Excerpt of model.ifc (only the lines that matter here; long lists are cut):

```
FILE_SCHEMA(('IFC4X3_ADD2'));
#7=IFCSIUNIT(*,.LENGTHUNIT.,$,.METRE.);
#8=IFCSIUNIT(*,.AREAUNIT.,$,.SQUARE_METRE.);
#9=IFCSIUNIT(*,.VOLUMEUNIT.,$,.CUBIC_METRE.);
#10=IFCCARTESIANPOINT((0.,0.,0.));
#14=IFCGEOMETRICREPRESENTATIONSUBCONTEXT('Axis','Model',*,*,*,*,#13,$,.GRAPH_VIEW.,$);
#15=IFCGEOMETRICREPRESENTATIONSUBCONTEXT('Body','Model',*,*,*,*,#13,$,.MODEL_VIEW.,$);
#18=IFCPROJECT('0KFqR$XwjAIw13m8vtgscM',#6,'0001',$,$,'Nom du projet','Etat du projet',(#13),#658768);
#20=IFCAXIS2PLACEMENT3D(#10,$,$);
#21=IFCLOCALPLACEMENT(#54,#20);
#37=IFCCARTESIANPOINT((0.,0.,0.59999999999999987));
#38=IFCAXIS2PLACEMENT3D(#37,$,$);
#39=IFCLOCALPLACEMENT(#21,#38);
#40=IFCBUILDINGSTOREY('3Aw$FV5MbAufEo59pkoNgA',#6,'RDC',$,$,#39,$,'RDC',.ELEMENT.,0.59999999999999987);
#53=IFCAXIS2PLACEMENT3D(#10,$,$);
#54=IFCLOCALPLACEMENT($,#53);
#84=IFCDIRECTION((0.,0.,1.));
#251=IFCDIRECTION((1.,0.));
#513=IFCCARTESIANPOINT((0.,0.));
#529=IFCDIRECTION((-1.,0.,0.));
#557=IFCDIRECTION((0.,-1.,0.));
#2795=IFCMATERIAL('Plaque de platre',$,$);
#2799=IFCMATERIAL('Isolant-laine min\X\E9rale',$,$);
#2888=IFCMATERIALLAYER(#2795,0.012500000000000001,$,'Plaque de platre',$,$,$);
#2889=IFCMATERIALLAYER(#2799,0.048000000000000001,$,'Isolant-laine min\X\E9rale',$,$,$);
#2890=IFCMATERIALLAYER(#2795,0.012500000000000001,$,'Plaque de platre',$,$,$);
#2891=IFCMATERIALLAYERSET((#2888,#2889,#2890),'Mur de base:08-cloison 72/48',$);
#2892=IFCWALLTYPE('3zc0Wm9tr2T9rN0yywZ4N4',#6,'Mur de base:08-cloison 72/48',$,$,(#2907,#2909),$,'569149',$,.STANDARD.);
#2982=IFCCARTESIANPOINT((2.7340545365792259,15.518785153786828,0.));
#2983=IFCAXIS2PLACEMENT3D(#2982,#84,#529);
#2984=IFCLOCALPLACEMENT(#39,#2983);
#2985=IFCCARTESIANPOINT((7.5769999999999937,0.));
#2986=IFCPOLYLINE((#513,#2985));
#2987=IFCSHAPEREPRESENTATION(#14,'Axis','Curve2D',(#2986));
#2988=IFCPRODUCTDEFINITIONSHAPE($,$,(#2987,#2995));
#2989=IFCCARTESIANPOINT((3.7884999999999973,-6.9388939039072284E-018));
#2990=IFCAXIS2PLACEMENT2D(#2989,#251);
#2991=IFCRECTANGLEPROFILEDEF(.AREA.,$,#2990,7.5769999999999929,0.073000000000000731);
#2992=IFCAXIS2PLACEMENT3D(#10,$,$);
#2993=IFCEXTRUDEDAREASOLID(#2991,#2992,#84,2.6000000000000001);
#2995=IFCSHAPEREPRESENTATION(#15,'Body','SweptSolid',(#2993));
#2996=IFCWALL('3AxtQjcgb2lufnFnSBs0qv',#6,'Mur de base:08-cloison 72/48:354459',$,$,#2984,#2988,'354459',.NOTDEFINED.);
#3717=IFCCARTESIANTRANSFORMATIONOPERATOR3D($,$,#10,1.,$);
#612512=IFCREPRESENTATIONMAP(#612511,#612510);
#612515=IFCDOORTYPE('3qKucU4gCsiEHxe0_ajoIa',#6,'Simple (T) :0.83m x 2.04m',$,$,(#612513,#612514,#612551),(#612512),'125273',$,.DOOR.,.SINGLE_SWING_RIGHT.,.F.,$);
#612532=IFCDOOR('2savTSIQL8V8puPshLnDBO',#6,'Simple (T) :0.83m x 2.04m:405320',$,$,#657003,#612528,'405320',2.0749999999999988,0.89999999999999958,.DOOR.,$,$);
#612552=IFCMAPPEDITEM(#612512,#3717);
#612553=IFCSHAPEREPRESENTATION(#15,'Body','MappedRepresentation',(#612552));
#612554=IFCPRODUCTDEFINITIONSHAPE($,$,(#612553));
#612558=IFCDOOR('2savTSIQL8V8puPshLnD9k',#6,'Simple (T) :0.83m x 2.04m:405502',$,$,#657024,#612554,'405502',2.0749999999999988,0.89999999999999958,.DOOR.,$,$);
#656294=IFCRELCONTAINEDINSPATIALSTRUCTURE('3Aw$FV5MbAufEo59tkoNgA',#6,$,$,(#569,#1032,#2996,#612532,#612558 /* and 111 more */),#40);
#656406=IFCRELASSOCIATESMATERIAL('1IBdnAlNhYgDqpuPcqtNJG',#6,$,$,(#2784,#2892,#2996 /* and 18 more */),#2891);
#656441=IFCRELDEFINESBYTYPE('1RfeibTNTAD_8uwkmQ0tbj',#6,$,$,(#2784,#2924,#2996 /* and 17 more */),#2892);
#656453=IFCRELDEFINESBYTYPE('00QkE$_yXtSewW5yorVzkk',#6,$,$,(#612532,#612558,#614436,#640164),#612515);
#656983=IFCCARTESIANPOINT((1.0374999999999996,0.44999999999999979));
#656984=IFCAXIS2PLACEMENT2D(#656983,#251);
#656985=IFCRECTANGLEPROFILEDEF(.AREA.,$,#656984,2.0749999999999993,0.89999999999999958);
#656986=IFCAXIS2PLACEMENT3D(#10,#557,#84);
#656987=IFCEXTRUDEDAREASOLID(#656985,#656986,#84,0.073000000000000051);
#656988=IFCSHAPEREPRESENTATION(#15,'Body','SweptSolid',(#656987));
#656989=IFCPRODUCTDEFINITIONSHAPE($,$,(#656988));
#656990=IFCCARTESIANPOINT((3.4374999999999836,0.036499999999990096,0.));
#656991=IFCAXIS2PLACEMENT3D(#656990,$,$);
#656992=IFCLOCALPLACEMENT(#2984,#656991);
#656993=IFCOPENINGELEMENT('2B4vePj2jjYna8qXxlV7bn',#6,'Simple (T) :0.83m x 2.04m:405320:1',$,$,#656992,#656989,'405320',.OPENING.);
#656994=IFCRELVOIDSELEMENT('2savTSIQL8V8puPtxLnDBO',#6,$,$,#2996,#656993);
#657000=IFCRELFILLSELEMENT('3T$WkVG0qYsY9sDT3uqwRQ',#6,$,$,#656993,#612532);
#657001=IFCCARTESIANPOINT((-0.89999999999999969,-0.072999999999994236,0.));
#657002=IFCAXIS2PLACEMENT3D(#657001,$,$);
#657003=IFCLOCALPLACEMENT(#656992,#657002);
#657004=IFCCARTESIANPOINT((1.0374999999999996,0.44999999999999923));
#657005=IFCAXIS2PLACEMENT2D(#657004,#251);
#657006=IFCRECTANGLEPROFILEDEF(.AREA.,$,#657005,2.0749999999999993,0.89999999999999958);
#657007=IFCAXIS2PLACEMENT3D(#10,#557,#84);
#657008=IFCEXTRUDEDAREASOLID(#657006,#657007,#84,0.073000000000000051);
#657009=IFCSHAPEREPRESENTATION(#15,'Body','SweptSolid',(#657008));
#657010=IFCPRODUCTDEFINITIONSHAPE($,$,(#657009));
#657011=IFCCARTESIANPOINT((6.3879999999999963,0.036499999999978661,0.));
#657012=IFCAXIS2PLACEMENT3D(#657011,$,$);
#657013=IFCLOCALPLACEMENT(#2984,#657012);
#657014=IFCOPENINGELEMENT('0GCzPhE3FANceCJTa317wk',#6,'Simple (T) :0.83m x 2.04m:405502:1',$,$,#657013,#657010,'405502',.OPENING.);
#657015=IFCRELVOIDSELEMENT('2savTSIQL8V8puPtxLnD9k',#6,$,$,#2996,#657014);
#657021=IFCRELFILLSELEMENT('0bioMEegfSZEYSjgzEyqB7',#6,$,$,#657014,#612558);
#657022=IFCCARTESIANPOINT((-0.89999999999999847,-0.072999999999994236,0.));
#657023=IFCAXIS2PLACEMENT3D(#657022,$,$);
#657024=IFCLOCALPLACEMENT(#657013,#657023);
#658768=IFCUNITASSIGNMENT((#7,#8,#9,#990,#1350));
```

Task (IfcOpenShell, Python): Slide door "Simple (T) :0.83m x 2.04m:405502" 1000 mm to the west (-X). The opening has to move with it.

```python
import ifcopenshell
import ifcopenshell.api.geometry
import ifcopenshell.util.placement

model = ifcopenshell.open("model.ifc")

door = model.by_id(612558)
opening = door.FillsVoids[0].RelatingOpeningElement
wall = opening.VoidsElements[0].RelatingBuildingElement

wall_matrix = ifcopenshell.util.placement.get_local_placement(wall.ObjectPlacement)
shift = wall_matrix[:3, 0] * 1.0
before = ifcopenshell.util.placement.get_local_placement(door.ObjectPlacement)[:3, 3].copy()

# The door is placed relative to its opening, so it follows when the opening moves.
matrix = ifcopenshell.util.placement.get_local_placement(opening.ObjectPlacement)
matrix[:3, 3] += shift
ifcopenshell.api.geometry.edit_object_placement(
    model, product=opening, matrix=matrix, is_si=False, should_transform_children=True
)

after = ifcopenshell.util.placement.get_local_placement(door.ObjectPlacement)[:3, 3]
print("door moved by", (after - before).round(3) + 0.0)

model.write("model_updated.ifc")
```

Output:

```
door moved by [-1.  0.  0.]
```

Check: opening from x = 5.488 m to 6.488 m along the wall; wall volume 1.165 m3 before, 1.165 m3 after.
